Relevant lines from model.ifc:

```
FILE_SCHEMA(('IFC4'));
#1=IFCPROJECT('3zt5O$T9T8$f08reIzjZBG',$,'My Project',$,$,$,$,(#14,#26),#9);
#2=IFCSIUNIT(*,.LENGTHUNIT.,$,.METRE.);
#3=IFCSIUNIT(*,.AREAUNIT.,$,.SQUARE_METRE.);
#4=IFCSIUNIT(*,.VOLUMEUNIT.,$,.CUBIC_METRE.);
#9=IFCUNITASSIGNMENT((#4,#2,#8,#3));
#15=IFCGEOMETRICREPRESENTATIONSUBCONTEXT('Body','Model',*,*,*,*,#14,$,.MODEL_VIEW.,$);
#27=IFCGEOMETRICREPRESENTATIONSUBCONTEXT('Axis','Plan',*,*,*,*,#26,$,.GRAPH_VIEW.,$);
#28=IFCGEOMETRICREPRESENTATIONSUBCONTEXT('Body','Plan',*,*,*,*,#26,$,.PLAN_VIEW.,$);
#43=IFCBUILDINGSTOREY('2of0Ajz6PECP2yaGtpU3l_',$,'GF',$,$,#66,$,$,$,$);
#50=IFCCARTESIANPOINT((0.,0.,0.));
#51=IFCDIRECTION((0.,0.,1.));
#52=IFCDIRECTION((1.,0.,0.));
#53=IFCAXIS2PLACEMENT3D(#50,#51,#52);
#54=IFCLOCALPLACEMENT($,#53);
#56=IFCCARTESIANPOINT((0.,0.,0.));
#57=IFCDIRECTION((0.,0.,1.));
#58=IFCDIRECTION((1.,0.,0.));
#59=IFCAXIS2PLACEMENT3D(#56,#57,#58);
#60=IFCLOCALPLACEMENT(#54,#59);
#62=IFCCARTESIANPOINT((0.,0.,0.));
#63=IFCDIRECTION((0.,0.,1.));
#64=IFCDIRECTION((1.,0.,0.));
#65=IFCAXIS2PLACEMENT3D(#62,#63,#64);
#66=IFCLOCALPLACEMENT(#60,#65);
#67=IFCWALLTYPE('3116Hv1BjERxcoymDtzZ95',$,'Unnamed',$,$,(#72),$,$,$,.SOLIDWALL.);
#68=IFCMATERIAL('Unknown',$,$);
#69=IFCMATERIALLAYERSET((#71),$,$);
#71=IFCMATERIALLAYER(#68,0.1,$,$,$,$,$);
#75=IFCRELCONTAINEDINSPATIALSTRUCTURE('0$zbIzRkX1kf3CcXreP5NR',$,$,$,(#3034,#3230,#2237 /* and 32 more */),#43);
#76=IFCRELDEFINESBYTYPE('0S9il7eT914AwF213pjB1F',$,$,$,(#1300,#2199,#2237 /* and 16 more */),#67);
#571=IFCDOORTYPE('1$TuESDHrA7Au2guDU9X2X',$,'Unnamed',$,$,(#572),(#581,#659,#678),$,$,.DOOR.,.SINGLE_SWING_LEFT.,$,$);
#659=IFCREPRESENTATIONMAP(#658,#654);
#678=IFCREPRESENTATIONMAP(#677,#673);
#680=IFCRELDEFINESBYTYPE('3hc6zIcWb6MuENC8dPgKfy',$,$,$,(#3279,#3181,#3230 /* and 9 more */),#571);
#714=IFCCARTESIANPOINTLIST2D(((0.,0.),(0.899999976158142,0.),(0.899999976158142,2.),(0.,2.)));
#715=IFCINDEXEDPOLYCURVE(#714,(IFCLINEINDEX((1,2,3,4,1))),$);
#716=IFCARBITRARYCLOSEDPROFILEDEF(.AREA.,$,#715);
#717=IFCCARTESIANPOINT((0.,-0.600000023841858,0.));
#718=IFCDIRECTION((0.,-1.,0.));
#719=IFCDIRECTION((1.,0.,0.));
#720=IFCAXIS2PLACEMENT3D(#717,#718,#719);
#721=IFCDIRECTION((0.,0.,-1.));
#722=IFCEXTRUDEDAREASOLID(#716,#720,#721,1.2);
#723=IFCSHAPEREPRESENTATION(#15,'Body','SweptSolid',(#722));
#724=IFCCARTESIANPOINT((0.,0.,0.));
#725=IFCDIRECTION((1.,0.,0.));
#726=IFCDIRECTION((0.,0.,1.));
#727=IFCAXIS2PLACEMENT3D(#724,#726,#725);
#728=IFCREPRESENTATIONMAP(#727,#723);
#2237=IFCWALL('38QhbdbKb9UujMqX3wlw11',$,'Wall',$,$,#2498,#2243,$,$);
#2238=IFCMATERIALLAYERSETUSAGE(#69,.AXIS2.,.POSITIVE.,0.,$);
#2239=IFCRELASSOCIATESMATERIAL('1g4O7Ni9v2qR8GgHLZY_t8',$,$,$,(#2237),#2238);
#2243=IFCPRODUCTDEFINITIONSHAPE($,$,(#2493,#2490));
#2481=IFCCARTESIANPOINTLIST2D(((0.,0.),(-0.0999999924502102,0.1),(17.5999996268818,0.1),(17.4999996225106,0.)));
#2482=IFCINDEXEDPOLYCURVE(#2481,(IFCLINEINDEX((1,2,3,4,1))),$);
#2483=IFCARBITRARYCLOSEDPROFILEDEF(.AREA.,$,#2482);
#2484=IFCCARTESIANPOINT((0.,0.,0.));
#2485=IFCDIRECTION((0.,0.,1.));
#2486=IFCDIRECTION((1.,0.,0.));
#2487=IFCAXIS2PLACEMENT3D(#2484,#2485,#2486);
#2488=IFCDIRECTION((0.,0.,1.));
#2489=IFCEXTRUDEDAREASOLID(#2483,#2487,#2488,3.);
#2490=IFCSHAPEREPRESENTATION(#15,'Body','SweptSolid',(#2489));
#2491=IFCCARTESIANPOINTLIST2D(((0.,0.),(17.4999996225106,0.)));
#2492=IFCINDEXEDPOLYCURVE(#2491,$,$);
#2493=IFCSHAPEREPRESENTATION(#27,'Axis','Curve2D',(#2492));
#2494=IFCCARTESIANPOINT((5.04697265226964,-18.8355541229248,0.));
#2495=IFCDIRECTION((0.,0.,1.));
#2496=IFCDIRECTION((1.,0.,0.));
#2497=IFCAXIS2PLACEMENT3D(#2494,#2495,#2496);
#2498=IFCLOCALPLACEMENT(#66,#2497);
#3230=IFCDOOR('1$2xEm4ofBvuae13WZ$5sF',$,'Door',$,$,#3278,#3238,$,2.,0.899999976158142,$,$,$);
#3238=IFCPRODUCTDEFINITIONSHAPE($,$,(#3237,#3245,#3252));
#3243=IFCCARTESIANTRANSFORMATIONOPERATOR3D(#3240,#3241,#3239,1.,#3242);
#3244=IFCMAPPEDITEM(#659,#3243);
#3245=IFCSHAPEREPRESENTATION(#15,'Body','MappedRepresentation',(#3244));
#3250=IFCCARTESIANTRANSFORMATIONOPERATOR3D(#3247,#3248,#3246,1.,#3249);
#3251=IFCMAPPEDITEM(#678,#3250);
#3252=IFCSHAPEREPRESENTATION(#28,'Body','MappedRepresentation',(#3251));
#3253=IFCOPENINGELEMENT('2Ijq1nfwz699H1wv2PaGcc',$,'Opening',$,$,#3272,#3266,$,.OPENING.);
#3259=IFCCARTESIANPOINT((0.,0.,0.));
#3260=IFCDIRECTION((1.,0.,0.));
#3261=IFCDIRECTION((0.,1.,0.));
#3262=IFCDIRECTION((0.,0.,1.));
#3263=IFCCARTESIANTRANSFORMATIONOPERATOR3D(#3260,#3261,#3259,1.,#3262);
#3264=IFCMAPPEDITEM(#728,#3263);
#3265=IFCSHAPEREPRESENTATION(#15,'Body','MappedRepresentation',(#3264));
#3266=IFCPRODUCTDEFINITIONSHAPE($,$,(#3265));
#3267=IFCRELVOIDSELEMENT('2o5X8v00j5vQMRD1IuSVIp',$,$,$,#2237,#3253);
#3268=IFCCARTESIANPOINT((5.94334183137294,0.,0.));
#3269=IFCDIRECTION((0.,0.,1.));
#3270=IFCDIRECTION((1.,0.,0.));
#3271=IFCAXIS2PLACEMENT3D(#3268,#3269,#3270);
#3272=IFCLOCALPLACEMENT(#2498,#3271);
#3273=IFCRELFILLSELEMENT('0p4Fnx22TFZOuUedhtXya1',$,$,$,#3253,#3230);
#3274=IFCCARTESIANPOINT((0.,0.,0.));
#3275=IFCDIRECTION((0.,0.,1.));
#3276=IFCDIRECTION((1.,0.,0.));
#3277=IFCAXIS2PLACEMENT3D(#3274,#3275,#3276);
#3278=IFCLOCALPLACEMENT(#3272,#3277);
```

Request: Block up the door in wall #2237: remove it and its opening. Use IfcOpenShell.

```python
import ifcopenshell
import ifcopenshell.api.feature
import ifcopenshell.api.root
import ifcopenshell.geom
import ifcopenshell.util.shape

model = ifcopenshell.open("model.ifc")
settings = ifcopenshell.geom.settings()


def volume(element):
    """Net volume in cubic metres, openings subtracted."""
    shape = ifcopenshell.geom.create_shape(settings, element)
    return ifcopenshell.util.shape.get_volume(shape.geometry)


door = model.by_id(3230)
opening = door.FillsVoids[0].RelatingOpeningElement
wall = opening.VoidsElements[0].RelatingBuildingElement
before = volume(wall)

ifcopenshell.api.root.remove_product(model, product=door)
ifcopenshell.api.feature.remove_feature(model, feature=opening)

after = volume(wall)

print(f"wall volume {before:.3f} -> {after:.3f} m3")

model.write("model_v2.ifc")
```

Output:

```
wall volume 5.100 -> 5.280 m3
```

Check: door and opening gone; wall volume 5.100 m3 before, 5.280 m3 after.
